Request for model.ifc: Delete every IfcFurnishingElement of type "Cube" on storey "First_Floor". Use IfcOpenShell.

First a look at what the model holds.

```python
import ifcopenshell
import ifcopenshell.util.element

model = ifcopenshell.open("model.ifc")
print(model.schema)
storey = next(s for s in model.by_type("IfcBuildingStorey") if s.Name == "First_Floor")
furniture = [e for e in ifcopenshell.util.element.get_decomposition(storey) if e.is_a("IfcFurnishingElement")]
seen = {}
for e in furniture:
    element_type = ifcopenshell.util.element.get_type(e)
    name = element_type.Name if element_type not in (None, e) else None
    seen[name] = seen.get(name, 0) + 1
for name, count in sorted(seen.items(), key=str):
    print(count, "x", name)
```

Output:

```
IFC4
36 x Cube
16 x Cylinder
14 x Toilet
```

```python
import ifcopenshell
import ifcopenshell.api.root
import ifcopenshell.util.element

model = ifcopenshell.open("model.ifc")

storey = next(s for s in model.by_type("IfcBuildingStorey") if s.Name == "First_Floor")
furniture = [e for e in ifcopenshell.util.element.get_decomposition(storey) if e.is_a("IfcFurnishingElement")]
targets = [e for e in furniture if (t := ifcopenshell.util.element.get_type(e)) not in (None, e) and t.Name == "Cube"]

for e in targets:
    ifcopenshell.api.root.remove_product(model, product=e)
print(len(targets), "removed")

model.write("model_rev.ifc")
```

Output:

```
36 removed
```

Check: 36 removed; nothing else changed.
